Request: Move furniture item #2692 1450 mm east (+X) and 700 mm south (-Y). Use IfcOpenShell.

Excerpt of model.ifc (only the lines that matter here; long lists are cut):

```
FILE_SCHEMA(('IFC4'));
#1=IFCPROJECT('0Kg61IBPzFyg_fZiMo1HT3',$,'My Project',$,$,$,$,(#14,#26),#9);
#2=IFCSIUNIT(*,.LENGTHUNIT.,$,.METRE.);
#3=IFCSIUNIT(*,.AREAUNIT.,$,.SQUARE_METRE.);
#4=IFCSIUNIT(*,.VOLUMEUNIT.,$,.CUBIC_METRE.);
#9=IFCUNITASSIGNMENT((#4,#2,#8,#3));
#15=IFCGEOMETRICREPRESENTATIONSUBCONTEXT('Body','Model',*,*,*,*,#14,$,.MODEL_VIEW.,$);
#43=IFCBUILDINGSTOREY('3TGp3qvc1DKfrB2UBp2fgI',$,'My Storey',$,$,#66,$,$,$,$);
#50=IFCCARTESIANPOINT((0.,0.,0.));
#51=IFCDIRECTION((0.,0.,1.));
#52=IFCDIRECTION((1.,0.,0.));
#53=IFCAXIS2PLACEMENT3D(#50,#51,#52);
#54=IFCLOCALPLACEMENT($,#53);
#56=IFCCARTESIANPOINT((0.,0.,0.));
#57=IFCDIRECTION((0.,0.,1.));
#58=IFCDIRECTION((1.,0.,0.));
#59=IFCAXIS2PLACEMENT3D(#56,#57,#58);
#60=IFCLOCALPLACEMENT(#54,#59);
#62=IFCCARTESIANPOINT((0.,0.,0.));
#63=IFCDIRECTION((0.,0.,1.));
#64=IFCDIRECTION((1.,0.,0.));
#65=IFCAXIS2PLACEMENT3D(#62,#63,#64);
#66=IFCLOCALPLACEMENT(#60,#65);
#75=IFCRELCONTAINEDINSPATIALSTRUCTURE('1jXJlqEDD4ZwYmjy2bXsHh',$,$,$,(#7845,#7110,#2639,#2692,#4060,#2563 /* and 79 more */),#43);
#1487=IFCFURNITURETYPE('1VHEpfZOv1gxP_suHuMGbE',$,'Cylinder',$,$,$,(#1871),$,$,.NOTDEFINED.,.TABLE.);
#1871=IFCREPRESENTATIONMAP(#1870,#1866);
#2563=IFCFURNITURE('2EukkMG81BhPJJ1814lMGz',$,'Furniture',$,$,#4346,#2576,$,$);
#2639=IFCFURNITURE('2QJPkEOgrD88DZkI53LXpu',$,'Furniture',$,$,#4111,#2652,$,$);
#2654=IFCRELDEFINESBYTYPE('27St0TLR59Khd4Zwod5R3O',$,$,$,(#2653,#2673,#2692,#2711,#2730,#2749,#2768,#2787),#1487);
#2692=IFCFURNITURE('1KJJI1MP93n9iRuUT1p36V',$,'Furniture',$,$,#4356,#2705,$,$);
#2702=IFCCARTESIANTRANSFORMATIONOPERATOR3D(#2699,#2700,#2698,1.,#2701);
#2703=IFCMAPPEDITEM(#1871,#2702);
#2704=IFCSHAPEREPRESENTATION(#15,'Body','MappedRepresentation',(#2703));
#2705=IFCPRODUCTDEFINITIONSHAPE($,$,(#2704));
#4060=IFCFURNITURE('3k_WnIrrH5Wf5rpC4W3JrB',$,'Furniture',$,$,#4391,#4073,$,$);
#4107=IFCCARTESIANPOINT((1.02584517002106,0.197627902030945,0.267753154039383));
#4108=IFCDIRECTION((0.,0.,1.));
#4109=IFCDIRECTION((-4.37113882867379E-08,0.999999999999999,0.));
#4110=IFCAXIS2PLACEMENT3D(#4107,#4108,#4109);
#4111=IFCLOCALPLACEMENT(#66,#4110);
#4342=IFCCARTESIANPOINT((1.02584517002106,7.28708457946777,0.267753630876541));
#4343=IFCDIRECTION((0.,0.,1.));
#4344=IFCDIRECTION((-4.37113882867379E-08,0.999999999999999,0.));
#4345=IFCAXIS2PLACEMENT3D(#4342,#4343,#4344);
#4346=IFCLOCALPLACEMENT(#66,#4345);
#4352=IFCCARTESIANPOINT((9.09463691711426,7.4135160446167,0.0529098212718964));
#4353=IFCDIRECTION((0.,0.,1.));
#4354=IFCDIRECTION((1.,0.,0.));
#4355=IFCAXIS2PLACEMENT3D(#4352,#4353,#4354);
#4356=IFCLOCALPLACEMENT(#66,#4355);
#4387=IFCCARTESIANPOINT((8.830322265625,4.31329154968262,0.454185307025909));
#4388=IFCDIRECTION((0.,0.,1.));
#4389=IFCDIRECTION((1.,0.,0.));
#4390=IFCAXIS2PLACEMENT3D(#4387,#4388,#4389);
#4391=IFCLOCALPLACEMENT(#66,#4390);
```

```python
import ifcopenshell
import ifcopenshell.api.geometry
import ifcopenshell.util.placement

model = ifcopenshell.open("model.ifc")

item = model.by_guid("1KJJI1MP93n9iRuUT1p36V")
matrix = ifcopenshell.util.placement.get_local_placement(item.ObjectPlacement)
matrix[0, 3] += 1.45
matrix[1, 3] -= 0.7
ifcopenshell.api.geometry.edit_object_placement(model, product=item, matrix=matrix, is_si=False)

print(ifcopenshell.util.placement.get_local_placement(item.ObjectPlacement).round(3) + 0.0)

model.write("model-out.ifc")
```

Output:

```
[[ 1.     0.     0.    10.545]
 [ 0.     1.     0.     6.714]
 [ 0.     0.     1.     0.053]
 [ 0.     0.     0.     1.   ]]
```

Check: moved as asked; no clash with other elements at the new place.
